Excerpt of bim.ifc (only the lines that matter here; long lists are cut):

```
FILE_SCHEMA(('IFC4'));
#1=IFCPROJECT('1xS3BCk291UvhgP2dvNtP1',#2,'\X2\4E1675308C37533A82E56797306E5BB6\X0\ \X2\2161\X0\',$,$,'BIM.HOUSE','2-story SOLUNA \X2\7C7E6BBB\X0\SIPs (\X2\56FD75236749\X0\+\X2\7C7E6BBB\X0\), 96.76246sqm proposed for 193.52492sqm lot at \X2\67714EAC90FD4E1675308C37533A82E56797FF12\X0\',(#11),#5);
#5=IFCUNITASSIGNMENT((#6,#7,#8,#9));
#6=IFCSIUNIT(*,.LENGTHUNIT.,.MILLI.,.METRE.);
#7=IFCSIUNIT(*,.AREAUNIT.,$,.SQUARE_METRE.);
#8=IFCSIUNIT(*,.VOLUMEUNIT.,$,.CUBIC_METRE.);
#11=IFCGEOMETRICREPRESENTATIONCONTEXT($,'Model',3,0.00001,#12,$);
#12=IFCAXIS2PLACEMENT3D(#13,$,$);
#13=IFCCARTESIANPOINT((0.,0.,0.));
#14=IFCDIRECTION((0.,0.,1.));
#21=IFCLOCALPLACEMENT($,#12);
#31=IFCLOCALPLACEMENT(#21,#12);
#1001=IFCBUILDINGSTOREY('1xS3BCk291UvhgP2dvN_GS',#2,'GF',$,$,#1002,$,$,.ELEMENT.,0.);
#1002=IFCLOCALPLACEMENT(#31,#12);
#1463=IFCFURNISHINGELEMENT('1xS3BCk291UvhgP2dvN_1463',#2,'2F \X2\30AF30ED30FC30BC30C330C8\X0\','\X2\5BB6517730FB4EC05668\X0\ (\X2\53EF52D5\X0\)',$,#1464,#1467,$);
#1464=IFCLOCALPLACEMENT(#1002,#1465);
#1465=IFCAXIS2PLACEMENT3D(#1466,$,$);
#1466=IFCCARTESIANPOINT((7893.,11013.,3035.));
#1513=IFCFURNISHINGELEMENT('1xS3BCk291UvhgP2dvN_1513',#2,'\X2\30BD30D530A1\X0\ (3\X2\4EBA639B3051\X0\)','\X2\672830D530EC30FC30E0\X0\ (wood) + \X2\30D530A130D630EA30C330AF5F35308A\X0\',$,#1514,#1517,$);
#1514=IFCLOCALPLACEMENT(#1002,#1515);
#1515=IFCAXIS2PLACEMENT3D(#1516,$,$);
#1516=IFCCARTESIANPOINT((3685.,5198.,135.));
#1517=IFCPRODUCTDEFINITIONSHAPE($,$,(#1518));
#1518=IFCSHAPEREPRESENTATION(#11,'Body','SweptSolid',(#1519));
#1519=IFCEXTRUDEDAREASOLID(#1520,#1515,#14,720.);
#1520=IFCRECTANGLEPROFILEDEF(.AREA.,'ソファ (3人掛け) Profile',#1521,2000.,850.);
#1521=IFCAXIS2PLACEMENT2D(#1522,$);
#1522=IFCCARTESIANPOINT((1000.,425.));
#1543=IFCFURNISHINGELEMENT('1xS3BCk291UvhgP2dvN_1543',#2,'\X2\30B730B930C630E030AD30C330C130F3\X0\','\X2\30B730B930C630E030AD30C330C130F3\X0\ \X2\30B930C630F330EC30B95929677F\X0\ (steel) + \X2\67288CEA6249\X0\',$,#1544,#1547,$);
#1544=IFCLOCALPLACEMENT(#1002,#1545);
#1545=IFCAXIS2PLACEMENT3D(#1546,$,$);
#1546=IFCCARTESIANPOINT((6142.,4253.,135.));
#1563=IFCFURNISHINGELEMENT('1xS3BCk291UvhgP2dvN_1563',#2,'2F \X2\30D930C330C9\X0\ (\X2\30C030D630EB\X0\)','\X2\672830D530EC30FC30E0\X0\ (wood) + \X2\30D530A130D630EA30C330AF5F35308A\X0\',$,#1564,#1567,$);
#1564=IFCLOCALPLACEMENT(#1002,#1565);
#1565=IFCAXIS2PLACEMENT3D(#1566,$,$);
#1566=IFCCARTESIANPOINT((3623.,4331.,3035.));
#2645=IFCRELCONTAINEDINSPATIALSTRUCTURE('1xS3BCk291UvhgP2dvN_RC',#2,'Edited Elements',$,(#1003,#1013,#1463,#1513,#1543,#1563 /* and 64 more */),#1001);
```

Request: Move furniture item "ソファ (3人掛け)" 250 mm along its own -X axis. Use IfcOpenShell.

```python
import ifcopenshell
import ifcopenshell.api.geometry
import ifcopenshell.util.placement
import ifcopenshell.util.unit

model = ifcopenshell.open("bim.ifc")
unit_scale = ifcopenshell.util.unit.calculate_unit_scale(model)

item = model.by_id(1513)
matrix = ifcopenshell.util.placement.get_local_placement(item.ObjectPlacement)
matrix[:3, 3] -= matrix[:3, 0] * 0.25 / unit_scale
ifcopenshell.api.geometry.edit_object_placement(model, product=item, matrix=matrix, is_si=False)

print(ifcopenshell.util.placement.get_local_placement(item.ObjectPlacement).round(3) + 0.0)

model.write("bim-out.ifc")
```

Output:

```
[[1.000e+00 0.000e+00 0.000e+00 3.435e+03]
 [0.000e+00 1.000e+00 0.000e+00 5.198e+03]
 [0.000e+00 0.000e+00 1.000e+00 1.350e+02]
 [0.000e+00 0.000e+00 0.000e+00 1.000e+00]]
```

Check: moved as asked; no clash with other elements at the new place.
